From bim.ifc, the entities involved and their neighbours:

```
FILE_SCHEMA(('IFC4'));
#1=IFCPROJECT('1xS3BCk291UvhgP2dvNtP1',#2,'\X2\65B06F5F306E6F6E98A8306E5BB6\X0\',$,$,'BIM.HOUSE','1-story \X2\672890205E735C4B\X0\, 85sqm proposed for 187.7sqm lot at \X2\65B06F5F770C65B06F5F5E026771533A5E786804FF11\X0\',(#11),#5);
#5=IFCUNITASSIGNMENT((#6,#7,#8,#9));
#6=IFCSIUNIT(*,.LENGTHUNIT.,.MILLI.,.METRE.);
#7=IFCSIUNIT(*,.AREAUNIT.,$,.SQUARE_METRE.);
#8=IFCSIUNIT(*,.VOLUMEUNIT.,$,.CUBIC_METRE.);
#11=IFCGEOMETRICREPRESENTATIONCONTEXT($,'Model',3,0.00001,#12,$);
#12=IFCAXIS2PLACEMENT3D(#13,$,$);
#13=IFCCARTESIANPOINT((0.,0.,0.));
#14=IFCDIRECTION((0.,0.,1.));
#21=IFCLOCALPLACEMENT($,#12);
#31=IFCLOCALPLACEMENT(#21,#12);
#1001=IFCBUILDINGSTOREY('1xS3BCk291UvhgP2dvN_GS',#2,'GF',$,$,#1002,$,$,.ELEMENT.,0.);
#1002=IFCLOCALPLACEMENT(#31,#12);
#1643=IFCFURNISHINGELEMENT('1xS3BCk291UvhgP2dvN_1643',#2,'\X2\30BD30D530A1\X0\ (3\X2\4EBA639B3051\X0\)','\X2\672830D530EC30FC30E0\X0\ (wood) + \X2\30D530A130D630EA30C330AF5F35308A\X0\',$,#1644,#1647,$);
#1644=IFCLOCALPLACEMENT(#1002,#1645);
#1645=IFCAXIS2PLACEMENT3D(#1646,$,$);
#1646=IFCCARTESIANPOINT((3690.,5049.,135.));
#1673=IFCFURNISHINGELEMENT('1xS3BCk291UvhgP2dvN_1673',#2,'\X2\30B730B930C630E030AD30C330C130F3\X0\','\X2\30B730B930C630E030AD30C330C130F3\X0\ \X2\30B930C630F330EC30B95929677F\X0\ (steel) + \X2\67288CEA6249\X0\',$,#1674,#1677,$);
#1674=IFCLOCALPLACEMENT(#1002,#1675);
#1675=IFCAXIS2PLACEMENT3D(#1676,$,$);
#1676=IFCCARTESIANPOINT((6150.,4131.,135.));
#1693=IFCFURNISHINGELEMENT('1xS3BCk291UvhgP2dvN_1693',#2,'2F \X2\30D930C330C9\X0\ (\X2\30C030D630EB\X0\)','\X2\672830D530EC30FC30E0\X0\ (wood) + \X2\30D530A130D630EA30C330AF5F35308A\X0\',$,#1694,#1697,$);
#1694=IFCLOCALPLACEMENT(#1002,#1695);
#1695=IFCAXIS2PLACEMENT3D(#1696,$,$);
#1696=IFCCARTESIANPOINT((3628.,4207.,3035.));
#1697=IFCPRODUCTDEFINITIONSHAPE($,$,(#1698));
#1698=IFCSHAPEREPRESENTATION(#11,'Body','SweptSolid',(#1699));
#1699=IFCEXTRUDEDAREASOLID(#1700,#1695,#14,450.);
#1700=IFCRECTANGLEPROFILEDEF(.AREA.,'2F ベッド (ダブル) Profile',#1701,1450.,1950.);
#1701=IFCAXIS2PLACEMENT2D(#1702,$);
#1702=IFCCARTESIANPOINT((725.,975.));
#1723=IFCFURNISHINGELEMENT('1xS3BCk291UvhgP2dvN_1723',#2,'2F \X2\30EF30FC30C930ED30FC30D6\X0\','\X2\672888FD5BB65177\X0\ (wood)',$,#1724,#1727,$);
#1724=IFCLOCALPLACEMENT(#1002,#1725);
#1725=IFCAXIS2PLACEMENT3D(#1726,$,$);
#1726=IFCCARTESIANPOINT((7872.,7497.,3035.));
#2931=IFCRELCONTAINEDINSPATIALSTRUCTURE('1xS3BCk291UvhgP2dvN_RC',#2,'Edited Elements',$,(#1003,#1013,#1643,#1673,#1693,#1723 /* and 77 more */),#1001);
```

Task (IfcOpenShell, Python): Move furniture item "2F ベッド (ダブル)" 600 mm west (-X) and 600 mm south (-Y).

```python
import ifcopenshell
import ifcopenshell.api.geometry
import ifcopenshell.util.placement
import ifcopenshell.util.unit

model = ifcopenshell.open("bim.ifc")
unit_scale = ifcopenshell.util.unit.calculate_unit_scale(model)

item = model.by_guid("1xS3BCk291UvhgP2dvN_1693")
matrix = ifcopenshell.util.placement.get_local_placement(item.ObjectPlacement)
matrix[0, 3] -= 0.6 / unit_scale
matrix[1, 3] -= 0.6 / unit_scale
ifcopenshell.api.geometry.edit_object_placement(model, product=item, matrix=matrix, is_si=False)

print(ifcopenshell.util.placement.get_local_placement(item.ObjectPlacement).round(3) + 0.0)

model.write("bim_updated.ifc")
```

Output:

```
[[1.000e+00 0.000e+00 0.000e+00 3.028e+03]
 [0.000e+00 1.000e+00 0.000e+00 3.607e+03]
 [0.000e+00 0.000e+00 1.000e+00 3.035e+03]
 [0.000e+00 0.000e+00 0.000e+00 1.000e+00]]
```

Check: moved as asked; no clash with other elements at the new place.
